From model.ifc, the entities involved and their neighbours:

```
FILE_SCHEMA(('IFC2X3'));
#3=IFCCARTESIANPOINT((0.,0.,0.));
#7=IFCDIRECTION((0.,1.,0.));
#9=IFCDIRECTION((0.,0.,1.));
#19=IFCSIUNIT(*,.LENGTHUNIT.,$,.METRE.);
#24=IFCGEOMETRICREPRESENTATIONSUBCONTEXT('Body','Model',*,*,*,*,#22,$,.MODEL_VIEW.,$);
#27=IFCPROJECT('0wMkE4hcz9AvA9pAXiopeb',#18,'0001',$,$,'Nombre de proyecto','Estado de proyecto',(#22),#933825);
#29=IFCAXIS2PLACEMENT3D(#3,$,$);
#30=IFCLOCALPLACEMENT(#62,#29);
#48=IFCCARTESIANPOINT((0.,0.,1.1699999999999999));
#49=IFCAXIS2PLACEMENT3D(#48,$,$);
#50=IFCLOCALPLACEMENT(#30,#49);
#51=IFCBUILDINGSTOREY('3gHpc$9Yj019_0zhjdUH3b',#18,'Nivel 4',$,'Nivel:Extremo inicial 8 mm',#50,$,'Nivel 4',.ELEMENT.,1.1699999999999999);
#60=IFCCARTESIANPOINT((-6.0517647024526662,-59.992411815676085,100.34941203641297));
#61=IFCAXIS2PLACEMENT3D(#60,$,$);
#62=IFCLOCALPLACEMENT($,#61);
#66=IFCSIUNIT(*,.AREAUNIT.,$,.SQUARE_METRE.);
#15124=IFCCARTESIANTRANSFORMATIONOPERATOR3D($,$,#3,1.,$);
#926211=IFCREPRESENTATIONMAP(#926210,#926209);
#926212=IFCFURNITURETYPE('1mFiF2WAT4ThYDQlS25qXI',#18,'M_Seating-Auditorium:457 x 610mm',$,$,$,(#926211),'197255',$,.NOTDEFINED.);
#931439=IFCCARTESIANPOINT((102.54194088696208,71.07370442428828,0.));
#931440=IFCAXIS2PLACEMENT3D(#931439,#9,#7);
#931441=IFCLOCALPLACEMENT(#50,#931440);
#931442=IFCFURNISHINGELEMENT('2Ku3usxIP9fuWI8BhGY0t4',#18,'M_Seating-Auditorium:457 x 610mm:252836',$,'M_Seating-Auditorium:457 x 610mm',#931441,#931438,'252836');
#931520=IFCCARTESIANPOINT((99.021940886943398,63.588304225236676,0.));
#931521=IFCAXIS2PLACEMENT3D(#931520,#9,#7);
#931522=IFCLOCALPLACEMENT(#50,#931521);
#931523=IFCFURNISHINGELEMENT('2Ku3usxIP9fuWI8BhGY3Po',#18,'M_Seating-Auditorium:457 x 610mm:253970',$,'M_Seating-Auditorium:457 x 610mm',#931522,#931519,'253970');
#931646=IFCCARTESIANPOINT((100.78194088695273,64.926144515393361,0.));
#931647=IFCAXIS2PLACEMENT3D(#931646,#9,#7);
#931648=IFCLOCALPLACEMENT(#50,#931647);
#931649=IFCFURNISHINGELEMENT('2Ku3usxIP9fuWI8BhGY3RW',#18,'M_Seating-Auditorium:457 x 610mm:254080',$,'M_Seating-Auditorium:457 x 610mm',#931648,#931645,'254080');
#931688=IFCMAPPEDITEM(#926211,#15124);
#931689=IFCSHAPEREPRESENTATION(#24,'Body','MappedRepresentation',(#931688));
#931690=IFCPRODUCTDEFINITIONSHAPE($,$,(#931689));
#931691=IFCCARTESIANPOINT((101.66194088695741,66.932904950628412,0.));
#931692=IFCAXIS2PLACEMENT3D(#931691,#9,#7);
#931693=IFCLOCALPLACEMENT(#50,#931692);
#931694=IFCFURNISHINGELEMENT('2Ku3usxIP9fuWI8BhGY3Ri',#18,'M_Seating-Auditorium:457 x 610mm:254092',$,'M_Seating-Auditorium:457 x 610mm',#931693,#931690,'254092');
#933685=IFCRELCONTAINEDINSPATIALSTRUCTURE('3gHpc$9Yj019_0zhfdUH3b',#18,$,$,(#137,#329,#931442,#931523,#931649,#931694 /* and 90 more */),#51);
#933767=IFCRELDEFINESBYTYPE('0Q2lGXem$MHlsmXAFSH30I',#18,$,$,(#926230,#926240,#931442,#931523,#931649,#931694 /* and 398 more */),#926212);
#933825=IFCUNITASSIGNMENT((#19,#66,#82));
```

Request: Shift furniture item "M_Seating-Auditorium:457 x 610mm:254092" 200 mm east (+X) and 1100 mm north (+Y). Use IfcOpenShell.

```python
import ifcopenshell
import ifcopenshell.api.geometry
import ifcopenshell.util.placement
import ifcopenshell.util.unit

model = ifcopenshell.open("model.ifc")
unit_scale = ifcopenshell.util.unit.calculate_unit_scale(model)

item = model.by_guid("2Ku3usxIP9fuWI8BhGY3Ri")
matrix = ifcopenshell.util.placement.get_local_placement(item.ObjectPlacement)
matrix[0, 3] += 0.2 / unit_scale
matrix[1, 3] += 1.1 / unit_scale
ifcopenshell.api.geometry.edit_object_placement(model, product=item, matrix=matrix, is_si=False)

print(ifcopenshell.util.placement.get_local_placement(item.ObjectPlacement).round(3) + 0.0)

model.write("model_edited.ifc")
```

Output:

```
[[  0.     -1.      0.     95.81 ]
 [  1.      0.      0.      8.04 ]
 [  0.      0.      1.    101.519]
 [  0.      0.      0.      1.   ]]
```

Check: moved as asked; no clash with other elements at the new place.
